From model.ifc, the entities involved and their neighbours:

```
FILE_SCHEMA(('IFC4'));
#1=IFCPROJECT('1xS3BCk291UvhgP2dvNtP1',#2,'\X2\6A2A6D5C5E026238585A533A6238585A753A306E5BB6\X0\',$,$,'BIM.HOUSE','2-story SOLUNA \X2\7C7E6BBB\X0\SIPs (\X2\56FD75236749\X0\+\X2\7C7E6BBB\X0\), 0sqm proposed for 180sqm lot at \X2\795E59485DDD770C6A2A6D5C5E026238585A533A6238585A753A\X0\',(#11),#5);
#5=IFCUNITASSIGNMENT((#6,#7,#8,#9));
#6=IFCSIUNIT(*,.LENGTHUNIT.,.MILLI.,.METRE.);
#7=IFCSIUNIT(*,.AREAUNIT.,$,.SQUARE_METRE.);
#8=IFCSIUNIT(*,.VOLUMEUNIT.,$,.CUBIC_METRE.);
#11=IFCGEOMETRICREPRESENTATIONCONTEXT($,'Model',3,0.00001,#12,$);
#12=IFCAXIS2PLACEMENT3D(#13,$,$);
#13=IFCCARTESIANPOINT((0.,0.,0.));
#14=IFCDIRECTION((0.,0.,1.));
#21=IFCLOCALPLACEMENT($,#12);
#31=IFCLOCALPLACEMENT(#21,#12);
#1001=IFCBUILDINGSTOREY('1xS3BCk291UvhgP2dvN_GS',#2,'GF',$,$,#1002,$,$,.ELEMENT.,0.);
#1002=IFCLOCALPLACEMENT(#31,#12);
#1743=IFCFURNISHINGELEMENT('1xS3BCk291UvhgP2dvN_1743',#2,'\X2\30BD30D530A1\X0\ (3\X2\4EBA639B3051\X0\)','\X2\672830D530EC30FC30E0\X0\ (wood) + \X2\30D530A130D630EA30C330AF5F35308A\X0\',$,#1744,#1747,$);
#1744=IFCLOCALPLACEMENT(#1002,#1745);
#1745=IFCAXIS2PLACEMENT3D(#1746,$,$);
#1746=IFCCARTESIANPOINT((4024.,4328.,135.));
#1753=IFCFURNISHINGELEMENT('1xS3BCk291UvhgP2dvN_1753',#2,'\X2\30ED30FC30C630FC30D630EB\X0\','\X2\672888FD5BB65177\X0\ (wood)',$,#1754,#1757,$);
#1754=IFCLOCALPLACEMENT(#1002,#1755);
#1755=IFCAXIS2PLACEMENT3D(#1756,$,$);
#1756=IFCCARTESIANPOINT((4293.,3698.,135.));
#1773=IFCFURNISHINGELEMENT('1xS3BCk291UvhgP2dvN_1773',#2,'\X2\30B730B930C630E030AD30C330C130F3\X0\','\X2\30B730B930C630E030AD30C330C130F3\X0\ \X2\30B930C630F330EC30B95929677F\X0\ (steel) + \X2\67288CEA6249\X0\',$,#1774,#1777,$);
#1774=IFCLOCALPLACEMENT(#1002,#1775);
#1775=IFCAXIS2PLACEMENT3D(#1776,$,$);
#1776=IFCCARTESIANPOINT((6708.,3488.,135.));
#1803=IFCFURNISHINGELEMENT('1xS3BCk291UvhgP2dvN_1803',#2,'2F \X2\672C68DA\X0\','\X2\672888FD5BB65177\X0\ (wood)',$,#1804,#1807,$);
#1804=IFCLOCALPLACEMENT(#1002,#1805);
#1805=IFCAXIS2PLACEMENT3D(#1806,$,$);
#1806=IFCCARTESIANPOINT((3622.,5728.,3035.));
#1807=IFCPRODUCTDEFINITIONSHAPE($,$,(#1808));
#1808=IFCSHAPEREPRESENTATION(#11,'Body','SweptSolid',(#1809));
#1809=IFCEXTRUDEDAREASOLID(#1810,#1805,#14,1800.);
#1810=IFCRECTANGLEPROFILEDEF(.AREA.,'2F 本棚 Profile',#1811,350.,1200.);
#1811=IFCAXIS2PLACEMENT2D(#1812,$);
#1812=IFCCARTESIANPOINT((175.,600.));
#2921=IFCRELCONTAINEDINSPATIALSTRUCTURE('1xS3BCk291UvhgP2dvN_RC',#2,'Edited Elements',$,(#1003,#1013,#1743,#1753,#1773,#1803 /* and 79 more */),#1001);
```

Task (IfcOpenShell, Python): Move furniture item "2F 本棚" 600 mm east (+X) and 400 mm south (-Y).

```python
import ifcopenshell
import ifcopenshell.api.geometry
import ifcopenshell.util.placement
import ifcopenshell.util.unit

model = ifcopenshell.open("model.ifc")
unit_scale = ifcopenshell.util.unit.calculate_unit_scale(model)

item = model.by_guid("1xS3BCk291UvhgP2dvN_1803")
matrix = ifcopenshell.util.placement.get_local_placement(item.ObjectPlacement)
matrix[0, 3] += 0.6 / unit_scale
matrix[1, 3] -= 0.4 / unit_scale
ifcopenshell.api.geometry.edit_object_placement(model, product=item, matrix=matrix, is_si=False)

print(ifcopenshell.util.placement.get_local_placement(item.ObjectPlacement).round(3) + 0.0)

model.write("model_updated.ifc")
```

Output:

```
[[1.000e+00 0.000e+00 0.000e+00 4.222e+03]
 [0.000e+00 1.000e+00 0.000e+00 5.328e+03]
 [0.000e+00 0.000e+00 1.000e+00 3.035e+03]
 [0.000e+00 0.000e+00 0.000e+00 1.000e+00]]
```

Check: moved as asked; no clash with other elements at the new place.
